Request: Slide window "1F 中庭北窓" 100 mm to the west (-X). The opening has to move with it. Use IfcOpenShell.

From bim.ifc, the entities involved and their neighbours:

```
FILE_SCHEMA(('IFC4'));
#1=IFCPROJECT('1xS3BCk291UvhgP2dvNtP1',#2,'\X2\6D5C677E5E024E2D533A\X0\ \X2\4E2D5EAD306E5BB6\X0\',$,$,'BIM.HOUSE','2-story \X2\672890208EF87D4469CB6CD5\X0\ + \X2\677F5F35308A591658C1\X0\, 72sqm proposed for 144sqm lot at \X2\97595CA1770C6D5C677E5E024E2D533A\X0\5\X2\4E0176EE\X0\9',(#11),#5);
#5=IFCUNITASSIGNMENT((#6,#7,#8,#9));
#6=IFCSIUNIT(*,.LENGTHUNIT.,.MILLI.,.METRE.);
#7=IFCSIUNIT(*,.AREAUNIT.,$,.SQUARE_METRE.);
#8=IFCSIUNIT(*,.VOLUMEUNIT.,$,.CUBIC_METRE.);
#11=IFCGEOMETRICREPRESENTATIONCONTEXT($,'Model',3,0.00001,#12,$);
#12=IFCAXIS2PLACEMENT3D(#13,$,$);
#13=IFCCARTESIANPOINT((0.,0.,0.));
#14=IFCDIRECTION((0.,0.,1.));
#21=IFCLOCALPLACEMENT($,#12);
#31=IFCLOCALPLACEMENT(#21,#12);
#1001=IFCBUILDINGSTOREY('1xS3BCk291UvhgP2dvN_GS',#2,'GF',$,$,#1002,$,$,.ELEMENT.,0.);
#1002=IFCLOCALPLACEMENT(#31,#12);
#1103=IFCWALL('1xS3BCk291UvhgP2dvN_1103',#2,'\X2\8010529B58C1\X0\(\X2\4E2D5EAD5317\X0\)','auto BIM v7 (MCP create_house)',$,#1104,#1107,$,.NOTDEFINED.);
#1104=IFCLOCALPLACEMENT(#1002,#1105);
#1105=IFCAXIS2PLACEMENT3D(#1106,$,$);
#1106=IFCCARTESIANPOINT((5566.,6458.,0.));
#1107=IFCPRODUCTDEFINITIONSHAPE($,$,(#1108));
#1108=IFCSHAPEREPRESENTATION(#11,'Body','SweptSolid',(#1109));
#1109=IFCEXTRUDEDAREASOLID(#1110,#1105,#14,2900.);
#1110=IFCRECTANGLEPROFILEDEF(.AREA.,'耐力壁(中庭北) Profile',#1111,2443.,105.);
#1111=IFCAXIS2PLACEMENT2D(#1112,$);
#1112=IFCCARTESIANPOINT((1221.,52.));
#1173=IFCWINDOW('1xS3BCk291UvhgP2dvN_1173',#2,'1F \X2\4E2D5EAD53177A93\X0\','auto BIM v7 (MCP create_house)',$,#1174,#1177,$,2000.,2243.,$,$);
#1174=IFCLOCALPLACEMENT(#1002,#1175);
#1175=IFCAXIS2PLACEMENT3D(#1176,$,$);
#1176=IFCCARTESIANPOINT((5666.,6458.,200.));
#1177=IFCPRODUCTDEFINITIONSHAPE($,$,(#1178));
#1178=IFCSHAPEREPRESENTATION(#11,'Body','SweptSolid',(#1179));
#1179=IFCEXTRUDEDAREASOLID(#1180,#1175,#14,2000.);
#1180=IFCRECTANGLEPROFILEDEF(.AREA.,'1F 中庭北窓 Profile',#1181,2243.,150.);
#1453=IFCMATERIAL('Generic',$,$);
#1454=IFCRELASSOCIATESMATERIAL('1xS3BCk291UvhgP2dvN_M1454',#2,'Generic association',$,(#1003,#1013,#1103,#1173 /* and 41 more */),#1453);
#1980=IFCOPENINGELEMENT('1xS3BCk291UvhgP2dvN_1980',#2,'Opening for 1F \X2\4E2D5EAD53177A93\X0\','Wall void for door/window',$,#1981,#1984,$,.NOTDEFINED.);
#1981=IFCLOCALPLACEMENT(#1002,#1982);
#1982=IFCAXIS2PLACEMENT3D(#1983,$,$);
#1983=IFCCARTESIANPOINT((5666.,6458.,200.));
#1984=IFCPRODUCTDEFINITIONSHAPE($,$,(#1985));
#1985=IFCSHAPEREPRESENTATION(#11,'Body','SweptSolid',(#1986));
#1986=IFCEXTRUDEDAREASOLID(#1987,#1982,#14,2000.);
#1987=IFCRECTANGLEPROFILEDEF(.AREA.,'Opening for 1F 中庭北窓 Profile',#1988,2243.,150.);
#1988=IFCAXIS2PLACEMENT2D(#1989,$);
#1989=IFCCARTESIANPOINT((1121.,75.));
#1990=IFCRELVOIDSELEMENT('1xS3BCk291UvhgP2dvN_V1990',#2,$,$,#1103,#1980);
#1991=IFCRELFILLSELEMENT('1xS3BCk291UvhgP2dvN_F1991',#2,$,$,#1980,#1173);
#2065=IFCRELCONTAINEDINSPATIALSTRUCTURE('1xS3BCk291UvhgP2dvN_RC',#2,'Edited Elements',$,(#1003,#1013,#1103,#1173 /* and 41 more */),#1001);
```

```python
import ifcopenshell
import ifcopenshell.api.geometry
import ifcopenshell.util.placement
import ifcopenshell.util.unit

model = ifcopenshell.open("bim.ifc")
unit_scale = ifcopenshell.util.unit.calculate_unit_scale(model)

window = model.by_id(1173)
opening = window.FillsVoids[0].RelatingOpeningElement
wall = opening.VoidsElements[0].RelatingBuildingElement

wall_matrix = ifcopenshell.util.placement.get_local_placement(wall.ObjectPlacement)
shift = wall_matrix[:3, 0] * -0.1 / unit_scale
before = ifcopenshell.util.placement.get_local_placement(window.ObjectPlacement)[:3, 3].copy()

# The window is not placed relative to its opening, so move both.
for product in (opening, window):
    matrix = ifcopenshell.util.placement.get_local_placement(product.ObjectPlacement)
    matrix[:3, 3] += shift
    ifcopenshell.api.geometry.edit_object_placement(model, product=product, matrix=matrix, is_si=False)

after = ifcopenshell.util.placement.get_local_placement(window.ObjectPlacement)[:3, 3]
print("window moved by", (after - before).round(3) + 0.0)

model.write("bim_updated.ifc")
```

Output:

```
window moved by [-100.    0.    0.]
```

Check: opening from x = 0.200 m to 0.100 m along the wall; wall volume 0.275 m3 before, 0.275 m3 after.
